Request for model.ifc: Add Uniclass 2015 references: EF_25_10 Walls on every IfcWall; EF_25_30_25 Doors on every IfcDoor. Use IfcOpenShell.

First a look at what the model holds.

```python
import ifcopenshell

model = ifcopenshell.open("model.ifc")
print(model.schema)
print("classifications:", [c.Name for c in model.by_type("IfcClassification")])
for ifc_class in ("IfcDoor", "IfcRoof", "IfcStair", "IfcWall", "IfcWindow"):
    print(ifc_class, len(model.by_type(ifc_class)))
```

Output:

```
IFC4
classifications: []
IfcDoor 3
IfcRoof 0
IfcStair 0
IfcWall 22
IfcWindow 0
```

```python
import ifcopenshell
import ifcopenshell.api.classification

model = ifcopenshell.open("model.ifc")

system = ifcopenshell.api.classification.add_classification(model, classification="Uniclass 2015")

codes = {
    "IfcWall": ("EF_25_10", "Walls"),
    "IfcDoor": ("EF_25_30_25", "Doors"),
}
for ifc_class, (code, name) in codes.items():
    products = model.by_type(ifc_class)
    ifcopenshell.api.classification.add_reference(
        model, products=products, classification=system, identification=code, name=name
    )
    print(code, len(products))

model.write("model_rev.ifc")
```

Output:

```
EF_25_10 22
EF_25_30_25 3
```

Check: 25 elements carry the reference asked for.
